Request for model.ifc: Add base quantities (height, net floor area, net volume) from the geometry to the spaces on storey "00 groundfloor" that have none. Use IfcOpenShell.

First a look at what the model holds.

```python
import ifcopenshell
import ifcopenshell.util.element
import ifcopenshell.util.unit

model = ifcopenshell.open("model.ifc")
print(model.schema)
for unit_type in ("LENGTHUNIT", "AREAUNIT", "VOLUMEUNIT"):
    print(unit_type, ifcopenshell.util.unit.calculate_unit_scale(model, unit_type))
storey = next(s for s in model.by_type("IfcBuildingStorey") if s.Name == "00 groundfloor")
spaces = [e for e in ifcopenshell.util.element.get_decomposition(storey) if e.is_a("IfcSpace")]
for e in sorted(spaces, key=lambda e: e.id()):
    print(e.id(), e.is_a(), e.Name, list(ifcopenshell.util.element.get_psets(e, qtos_only=True)), sep=" | ")
```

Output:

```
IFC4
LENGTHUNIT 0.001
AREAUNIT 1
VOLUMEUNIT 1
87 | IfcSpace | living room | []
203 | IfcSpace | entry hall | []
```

```python
import ifcopenshell
import ifcopenshell.api.pset
import ifcopenshell.geom
import ifcopenshell.util.element
import ifcopenshell.util.shape
import ifcopenshell.util.unit

model = ifcopenshell.open("model.ifc")
unit_scale = ifcopenshell.util.unit.calculate_unit_scale(model)
area_scale = ifcopenshell.util.unit.calculate_unit_scale(model, "AREAUNIT")
volume_scale = ifcopenshell.util.unit.calculate_unit_scale(model, "VOLUMEUNIT")
settings = ifcopenshell.geom.settings()

storey = next(s for s in model.by_type("IfcBuildingStorey") if s.Name == "00 groundfloor")
spaces = [e for e in ifcopenshell.util.element.get_decomposition(storey) if e.is_a("IfcSpace")]

for e in sorted(spaces, key=lambda e: e.id()):
    if ifcopenshell.util.element.get_psets(e, qtos_only=True, should_inherit=False):
        continue
    # Geometry comes back in metres, in the element's own axes.
    shape = ifcopenshell.geom.create_shape(settings, e)
    values = {
        "Height": ifcopenshell.util.shape.get_z(shape.geometry) / unit_scale,
        "NetFloorArea": ifcopenshell.util.shape.get_footprint_area(shape.geometry) / area_scale,
        "NetVolume": ifcopenshell.util.shape.get_volume(shape.geometry) / volume_scale,
    }
    qto = ifcopenshell.api.pset.add_qto(model, product=e, name="Qto_SpaceBaseQuantities")
    ifcopenshell.api.pset.edit_qto(model, qto=qto, properties=values)
    print(e.id(), {k: round(v, 3) for k, v in values.items()})

model.write("model_edited.ifc")
```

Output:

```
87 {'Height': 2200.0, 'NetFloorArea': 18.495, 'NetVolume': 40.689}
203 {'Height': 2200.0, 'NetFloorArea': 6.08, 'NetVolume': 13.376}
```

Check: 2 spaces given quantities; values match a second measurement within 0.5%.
